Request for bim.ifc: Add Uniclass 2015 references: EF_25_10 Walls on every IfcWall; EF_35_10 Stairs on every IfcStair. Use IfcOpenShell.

First a look at what the model holds.

```python
import ifcopenshell

model = ifcopenshell.open("bim.ifc")
print(model.schema)
print("classifications:", [c.Name for c in model.by_type("IfcClassification")])
for ifc_class in ("IfcDoor", "IfcRoof", "IfcStair", "IfcWall", "IfcWindow"):
    print(ifc_class, len(model.by_type(ifc_class)))
```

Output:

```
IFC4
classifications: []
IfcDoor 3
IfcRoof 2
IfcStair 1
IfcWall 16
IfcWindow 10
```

```python
import ifcopenshell
import ifcopenshell.api.classification

model = ifcopenshell.open("bim.ifc")

system = ifcopenshell.api.classification.add_classification(model, classification="Uniclass 2015")

codes = {
    "IfcWall": ("EF_25_10", "Walls"),
    "IfcStair": ("EF_35_10", "Stairs"),
}
for ifc_class, (code, name) in codes.items():
    products = model.by_type(ifc_class)
    ifcopenshell.api.classification.add_reference(
        model, products=products, classification=system, identification=code, name=name
    )
    print(code, len(products))

model.write("bim_v2.ifc")
```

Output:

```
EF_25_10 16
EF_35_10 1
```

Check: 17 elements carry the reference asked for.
